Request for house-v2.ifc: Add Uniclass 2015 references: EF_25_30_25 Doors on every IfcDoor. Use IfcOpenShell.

First a look at what the model holds.

```python
import ifcopenshell

model = ifcopenshell.open("house-v2.ifc")
print(model.schema)
print("classifications:", [c.Name for c in model.by_type("IfcClassification")])
for ifc_class in ("IfcDoor", "IfcRoof", "IfcStair", "IfcWall", "IfcWindow"):
    print(ifc_class, len(model.by_type(ifc_class)))
```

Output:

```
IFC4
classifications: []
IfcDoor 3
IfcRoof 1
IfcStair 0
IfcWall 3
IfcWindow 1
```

```python
import ifcopenshell
import ifcopenshell.api.classification

model = ifcopenshell.open("house-v2.ifc")

system = ifcopenshell.api.classification.add_classification(model, classification="Uniclass 2015")

codes = {
    "IfcDoor": ("EF_25_30_25", "Doors"),
}
for ifc_class, (code, name) in codes.items():
    products = model.by_type(ifc_class)
    ifcopenshell.api.classification.add_reference(
        model, products=products, classification=system, identification=code, name=name
    )
    print(code, len(products))

model.write("house-v2_rev.ifc")
```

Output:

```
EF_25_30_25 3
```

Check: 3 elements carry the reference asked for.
